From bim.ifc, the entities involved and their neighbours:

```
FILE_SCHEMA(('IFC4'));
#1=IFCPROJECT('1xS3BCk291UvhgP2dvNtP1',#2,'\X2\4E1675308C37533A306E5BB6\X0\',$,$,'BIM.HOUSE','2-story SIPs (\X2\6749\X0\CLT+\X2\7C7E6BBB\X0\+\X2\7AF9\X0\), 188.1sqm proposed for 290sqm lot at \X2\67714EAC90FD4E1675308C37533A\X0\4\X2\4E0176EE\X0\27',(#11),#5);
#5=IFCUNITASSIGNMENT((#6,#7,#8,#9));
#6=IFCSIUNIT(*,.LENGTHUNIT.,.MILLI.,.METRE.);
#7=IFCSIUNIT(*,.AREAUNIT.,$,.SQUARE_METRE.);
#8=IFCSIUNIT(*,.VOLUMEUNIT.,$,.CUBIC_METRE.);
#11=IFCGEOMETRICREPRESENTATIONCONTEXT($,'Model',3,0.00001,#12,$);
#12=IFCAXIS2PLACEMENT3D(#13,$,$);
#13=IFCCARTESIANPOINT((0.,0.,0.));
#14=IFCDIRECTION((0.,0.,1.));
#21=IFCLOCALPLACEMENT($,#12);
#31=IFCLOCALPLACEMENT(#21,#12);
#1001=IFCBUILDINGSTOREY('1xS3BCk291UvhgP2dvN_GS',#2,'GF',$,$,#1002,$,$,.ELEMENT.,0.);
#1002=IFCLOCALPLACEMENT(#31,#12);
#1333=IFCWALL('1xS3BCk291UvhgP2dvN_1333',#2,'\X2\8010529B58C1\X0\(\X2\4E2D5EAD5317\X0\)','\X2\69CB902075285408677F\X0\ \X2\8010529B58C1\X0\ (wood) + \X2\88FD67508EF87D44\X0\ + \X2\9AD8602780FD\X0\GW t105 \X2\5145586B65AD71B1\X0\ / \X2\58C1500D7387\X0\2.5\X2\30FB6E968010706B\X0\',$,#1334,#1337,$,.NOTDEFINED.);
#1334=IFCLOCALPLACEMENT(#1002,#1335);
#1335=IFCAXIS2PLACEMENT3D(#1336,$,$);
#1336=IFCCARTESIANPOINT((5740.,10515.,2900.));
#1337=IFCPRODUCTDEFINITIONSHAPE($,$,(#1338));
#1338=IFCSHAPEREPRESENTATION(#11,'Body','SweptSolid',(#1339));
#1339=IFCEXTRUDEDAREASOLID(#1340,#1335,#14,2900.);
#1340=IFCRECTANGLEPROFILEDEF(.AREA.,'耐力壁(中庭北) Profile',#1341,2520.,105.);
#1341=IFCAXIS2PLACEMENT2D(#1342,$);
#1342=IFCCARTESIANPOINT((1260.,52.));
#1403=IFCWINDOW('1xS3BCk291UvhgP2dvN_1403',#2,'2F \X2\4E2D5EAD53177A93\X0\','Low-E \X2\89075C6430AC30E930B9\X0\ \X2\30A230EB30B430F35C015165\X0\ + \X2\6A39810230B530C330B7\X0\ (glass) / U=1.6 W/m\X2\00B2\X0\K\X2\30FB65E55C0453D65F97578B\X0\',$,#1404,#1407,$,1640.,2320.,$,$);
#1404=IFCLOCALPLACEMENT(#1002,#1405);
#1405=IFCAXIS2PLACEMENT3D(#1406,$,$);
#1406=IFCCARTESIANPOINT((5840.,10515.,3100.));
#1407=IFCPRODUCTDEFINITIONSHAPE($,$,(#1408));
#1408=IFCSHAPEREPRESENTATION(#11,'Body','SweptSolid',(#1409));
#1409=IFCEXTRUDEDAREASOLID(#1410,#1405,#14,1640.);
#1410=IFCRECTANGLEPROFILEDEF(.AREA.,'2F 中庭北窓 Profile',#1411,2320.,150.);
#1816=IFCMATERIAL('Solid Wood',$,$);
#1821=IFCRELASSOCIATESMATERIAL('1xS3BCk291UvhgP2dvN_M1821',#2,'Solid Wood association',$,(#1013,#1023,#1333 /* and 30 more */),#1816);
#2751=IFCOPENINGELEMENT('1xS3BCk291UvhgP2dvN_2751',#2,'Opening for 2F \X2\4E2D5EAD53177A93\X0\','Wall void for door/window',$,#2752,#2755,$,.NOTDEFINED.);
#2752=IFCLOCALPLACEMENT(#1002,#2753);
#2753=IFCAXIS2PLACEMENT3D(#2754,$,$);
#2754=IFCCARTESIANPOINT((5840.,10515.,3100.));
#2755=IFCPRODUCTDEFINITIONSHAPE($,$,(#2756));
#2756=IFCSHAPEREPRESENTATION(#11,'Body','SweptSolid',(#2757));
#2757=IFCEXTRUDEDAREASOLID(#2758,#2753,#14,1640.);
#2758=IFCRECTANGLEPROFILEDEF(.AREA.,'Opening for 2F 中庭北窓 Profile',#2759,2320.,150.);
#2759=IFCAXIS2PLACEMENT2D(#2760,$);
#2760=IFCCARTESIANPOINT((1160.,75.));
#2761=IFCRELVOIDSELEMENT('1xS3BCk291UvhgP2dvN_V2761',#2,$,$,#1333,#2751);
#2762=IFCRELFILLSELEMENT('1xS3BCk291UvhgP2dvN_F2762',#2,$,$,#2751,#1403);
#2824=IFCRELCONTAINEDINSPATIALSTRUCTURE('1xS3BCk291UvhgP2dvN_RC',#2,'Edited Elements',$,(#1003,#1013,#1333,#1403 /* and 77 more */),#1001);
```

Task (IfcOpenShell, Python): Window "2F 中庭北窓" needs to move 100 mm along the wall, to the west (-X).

```python
import ifcopenshell
import ifcopenshell.api.geometry
import ifcopenshell.util.placement
import ifcopenshell.util.unit

model = ifcopenshell.open("bim.ifc")
unit_scale = ifcopenshell.util.unit.calculate_unit_scale(model)

window = model.by_guid("1xS3BCk291UvhgP2dvN_1403")
opening = window.FillsVoids[0].RelatingOpeningElement
wall = opening.VoidsElements[0].RelatingBuildingElement

wall_matrix = ifcopenshell.util.placement.get_local_placement(wall.ObjectPlacement)
shift = wall_matrix[:3, 0] * -0.1 / unit_scale
before = ifcopenshell.util.placement.get_local_placement(window.ObjectPlacement)[:3, 3].copy()

# The window is not placed relative to its opening, so move both.
for product in (opening, window):
    matrix = ifcopenshell.util.placement.get_local_placement(product.ObjectPlacement)
    matrix[:3, 3] += shift
    ifcopenshell.api.geometry.edit_object_placement(model, product=product, matrix=matrix, is_si=False)

after = ifcopenshell.util.placement.get_local_placement(window.ObjectPlacement)[:3, 3]
print("window moved by", (after - before).round(3) + 0.0)

model.write("bim_rev.ifc")
```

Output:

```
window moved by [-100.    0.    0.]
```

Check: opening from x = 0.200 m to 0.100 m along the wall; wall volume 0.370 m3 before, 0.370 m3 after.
